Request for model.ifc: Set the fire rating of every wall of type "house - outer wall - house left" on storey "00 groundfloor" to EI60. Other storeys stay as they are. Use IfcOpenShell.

First a look at what the model holds.

```python
import ifcopenshell
import ifcopenshell.util.element

model = ifcopenshell.open("model.ifc")
print(model.schema)
storey = next(s for s in model.by_type("IfcBuildingStorey") if s.Name == "00 groundfloor")
walls = [e for e in ifcopenshell.util.element.get_decomposition(storey) if e.is_a("IfcWall")]
seen = {}
for e in walls:
    element_type = ifcopenshell.util.element.get_type(e)
    key = (element_type.Name if element_type != e and element_type else None, ifcopenshell.util.element.get_pset(e, "Pset_WallCommon", "FireRating"))
    seen[key] = seen.get(key, 0) + 1
for (name, value), count in sorted(seen.items(), key=str):
    print(count, "x", name, "|", value)
```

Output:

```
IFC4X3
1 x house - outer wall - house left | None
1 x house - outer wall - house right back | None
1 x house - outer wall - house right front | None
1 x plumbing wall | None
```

```python
import ifcopenshell
import ifcopenshell.api.pset
import ifcopenshell.util.element

model = ifcopenshell.open("model.ifc")

storey = next(s for s in model.by_type("IfcBuildingStorey") if s.Name == "00 groundfloor")
walls = [e for e in ifcopenshell.util.element.get_decomposition(storey) if e.is_a("IfcWall")]

count = 0
for e in walls:
    element_type = ifcopenshell.util.element.get_type(e)
    if element_type in (None, e) or element_type.Name != "house - outer wall - house left":
        continue
    # add_pset returns the element's existing set when there is one.
    pset = ifcopenshell.api.pset.add_pset(model, product=e, name="Pset_WallCommon")
    ifcopenshell.api.pset.edit_pset(model, pset=pset, properties={"FireRating": "EI60"})
    count += 1

print(count, "walls updated")

model.write("model_updated.ifc")
```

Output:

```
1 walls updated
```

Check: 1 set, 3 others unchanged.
